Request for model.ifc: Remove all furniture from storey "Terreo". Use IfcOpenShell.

First a look at what the model holds.

```python
import ifcopenshell
import ifcopenshell.util.element

model = ifcopenshell.open("model.ifc")
print(model.schema)
storey = next(s for s in model.by_type("IfcBuildingStorey") if s.Name == "Terreo")
furniture = [e for e in ifcopenshell.util.element.get_decomposition(storey) if e.is_a("IfcFurnishingElement")]
seen = {}
for e in furniture:
    element_type = ifcopenshell.util.element.get_type(e)
    name = element_type.Name if element_type not in (None, e) else None
    seen[name] = seen.get(name, 0) + 1
for name, count in sorted(seen.items(), key=str):
    print(count, "x", name)
```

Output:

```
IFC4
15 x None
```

```python
import ifcopenshell
import ifcopenshell.api.root
import ifcopenshell.util.element

model = ifcopenshell.open("model.ifc")

storey = next(s for s in model.by_type("IfcBuildingStorey") if s.Name == "Terreo")
furniture = [e for e in ifcopenshell.util.element.get_decomposition(storey) if e.is_a("IfcFurnishingElement")]

for e in furniture:
    ifcopenshell.api.root.remove_product(model, product=e)
print(len(furniture), "removed")

model.write("model_v2.ifc")
```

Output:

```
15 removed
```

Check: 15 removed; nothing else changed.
